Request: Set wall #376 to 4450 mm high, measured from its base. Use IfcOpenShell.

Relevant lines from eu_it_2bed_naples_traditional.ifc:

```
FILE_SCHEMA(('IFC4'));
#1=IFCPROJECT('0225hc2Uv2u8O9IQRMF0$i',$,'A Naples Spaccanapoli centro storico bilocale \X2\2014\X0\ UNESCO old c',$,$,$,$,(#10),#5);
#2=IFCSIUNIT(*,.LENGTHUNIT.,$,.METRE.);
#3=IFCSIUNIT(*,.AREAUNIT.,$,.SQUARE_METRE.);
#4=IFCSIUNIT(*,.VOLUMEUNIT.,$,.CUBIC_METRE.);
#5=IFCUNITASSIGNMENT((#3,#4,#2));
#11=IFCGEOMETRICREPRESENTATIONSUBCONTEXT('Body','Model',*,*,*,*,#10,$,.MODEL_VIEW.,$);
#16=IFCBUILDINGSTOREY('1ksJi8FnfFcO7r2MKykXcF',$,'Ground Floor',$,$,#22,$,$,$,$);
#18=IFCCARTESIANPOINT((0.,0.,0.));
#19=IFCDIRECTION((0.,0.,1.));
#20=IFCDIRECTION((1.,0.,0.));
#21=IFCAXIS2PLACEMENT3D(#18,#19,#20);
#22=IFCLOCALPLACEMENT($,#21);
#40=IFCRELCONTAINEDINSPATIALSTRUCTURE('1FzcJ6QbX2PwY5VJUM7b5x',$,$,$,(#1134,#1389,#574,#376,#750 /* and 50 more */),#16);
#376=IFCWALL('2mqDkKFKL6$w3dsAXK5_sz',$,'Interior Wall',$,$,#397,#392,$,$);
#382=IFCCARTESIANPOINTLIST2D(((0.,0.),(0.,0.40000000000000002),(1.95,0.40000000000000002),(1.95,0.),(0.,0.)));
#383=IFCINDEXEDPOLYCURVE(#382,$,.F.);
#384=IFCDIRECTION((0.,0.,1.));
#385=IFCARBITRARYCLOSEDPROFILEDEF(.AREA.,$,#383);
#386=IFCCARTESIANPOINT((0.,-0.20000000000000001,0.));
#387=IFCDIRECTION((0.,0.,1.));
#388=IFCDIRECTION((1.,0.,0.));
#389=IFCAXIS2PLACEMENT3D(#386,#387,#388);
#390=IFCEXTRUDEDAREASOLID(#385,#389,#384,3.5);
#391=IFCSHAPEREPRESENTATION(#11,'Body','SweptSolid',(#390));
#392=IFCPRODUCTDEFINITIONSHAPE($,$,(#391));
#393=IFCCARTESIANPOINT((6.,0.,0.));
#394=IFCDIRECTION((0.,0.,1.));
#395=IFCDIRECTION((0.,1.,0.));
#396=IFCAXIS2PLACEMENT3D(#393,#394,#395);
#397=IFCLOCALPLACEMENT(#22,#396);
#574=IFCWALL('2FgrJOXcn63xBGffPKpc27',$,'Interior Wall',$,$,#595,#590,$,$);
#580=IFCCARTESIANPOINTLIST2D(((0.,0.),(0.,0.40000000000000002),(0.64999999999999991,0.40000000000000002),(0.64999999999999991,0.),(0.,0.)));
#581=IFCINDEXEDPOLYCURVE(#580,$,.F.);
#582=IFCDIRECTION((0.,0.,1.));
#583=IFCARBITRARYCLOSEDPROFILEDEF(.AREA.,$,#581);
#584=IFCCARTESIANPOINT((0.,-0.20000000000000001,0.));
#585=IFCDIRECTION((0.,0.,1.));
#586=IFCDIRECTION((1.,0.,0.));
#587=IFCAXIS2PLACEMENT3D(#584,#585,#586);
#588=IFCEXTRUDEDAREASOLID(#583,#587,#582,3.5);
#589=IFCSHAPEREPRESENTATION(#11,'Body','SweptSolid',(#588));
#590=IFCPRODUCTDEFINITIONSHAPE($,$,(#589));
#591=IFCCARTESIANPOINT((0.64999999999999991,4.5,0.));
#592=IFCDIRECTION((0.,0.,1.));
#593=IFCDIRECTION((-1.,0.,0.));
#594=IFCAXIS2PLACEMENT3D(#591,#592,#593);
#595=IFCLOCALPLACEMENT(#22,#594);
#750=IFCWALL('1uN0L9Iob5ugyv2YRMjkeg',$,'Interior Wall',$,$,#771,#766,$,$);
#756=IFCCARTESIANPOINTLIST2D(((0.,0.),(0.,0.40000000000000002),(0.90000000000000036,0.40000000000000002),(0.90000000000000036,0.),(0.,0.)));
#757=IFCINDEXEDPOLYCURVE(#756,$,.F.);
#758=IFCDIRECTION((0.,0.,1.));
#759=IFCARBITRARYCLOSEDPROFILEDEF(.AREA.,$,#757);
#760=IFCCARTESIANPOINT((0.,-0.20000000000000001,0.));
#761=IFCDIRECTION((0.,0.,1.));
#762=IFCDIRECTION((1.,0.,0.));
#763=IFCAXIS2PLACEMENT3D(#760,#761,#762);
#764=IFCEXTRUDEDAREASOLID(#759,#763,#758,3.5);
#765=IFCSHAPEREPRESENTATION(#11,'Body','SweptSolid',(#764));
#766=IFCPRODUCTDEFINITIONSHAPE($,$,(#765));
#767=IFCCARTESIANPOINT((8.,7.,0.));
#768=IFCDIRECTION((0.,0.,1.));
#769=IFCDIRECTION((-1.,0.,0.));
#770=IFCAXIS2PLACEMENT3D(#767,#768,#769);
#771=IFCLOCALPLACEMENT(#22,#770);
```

```python
import ifcopenshell
import ifcopenshell.geom
import ifcopenshell.util.representation
import ifcopenshell.util.shape

model = ifcopenshell.open("eu_it_2bed_naples_traditional.ifc")
settings = ifcopenshell.geom.settings()


def volume(element):
    """Net volume in cubic metres, openings subtracted."""
    shape = ifcopenshell.geom.create_shape(settings, element)
    return ifcopenshell.util.shape.get_volume(shape.geometry)


wall = model.by_guid("2mqDkKFKL6$w3dsAXK5_sz")
before = volume(wall)

body = ifcopenshell.util.representation.get_representation(wall, "Model", "Body")
solid = body.Items[0]
old_height = solid.Depth
solid.Depth = 4.45
after = volume(wall)

print(f"height {old_height:g} -> {solid.Depth:g}, volume {before:.3f} -> {after:.3f} m3")

model.write("eu_it_2bed_naples_traditional-out.ifc")
```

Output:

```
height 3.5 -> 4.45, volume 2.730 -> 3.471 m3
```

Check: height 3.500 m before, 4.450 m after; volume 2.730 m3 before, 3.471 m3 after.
